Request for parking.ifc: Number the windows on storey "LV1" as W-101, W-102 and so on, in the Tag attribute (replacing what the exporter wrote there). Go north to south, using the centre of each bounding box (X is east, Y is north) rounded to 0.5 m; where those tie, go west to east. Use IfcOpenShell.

First a look at what the model holds.

```python
import ifcopenshell
import ifcopenshell.util.element
import ifcopenshell.util.placement

model = ifcopenshell.open("parking.ifc")
print(model.schema)
storey = next(s for s in model.by_type("IfcBuildingStorey") if s.Name == "LV1")
windows = [e for e in ifcopenshell.util.element.get_decomposition(storey) if e.is_a("IfcWindow")]
for e in sorted(windows, key=lambda e: e.id()):
    origin = ifcopenshell.util.placement.get_local_placement(e.ObjectPlacement)[:3, 3]
    print(e.id(), e.Tag, e.Name, origin.round(2) + 0.0, sep=" | ")
```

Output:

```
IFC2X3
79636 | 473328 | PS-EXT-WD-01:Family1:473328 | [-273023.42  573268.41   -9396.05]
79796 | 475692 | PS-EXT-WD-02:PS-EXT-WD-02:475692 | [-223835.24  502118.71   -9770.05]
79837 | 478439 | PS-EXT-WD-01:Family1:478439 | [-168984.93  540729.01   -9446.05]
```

```python
import ifcopenshell
import ifcopenshell.geom
import ifcopenshell.util.element
import ifcopenshell.util.shape

model = ifcopenshell.open("parking.ifc")
settings = ifcopenshell.geom.settings()
settings.set("use-world-coords", True)


def centre(element):
    shape = ifcopenshell.geom.create_shape(settings, element)
    return ifcopenshell.util.shape.get_bbox_centroid(shape.geometry)


storey = next(s for s in model.by_type("IfcBuildingStorey") if s.Name == "LV1")
windows = [e for e in ifcopenshell.util.element.get_decomposition(storey) if e.is_a("IfcWindow")]

# Insertion points can sit at a corner or the storey origin, so sort by the geometry (in metres).
centres = {e: centre(e) for e in windows}
windows.sort(key=lambda e: (-round(centres[e][1] / 0.5), centres[e][0]))

for i, e in enumerate(windows, start=1):
    number = f"W-1{i:02d}"
    e.Tag = number
    print(e.id(), number)

model.write("parking_updated.ifc")
```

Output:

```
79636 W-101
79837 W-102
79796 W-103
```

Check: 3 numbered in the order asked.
